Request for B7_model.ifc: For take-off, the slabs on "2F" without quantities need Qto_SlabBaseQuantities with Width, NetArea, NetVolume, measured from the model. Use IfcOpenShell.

First a look at what the model holds.

```python
import ifcopenshell
import ifcopenshell.util.element
import ifcopenshell.util.unit

model = ifcopenshell.open("B7_model.ifc")
print(model.schema)
for unit_type in ("LENGTHUNIT", "AREAUNIT", "VOLUMEUNIT"):
    print(unit_type, ifcopenshell.util.unit.calculate_unit_scale(model, unit_type))
storey = next(s for s in model.by_type("IfcBuildingStorey") if s.Name == "2F")
slabs = [e for e in ifcopenshell.util.element.get_decomposition(storey) if e.is_a("IfcSlab")]
for e in sorted(slabs, key=lambda e: e.id()):
    print(e.id(), e.is_a(), e.Name, list(ifcopenshell.util.element.get_psets(e, qtos_only=True)), sep=" | ")
```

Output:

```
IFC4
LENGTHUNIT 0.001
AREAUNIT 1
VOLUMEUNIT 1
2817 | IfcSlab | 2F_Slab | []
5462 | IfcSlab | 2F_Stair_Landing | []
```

```python
import ifcopenshell
import ifcopenshell.api.pset
import ifcopenshell.geom
import ifcopenshell.util.element
import ifcopenshell.util.shape
import ifcopenshell.util.unit

model = ifcopenshell.open("B7_model.ifc")
unit_scale = ifcopenshell.util.unit.calculate_unit_scale(model)
area_scale = ifcopenshell.util.unit.calculate_unit_scale(model, "AREAUNIT")
volume_scale = ifcopenshell.util.unit.calculate_unit_scale(model, "VOLUMEUNIT")
settings = ifcopenshell.geom.settings()

storey = next(s for s in model.by_type("IfcBuildingStorey") if s.Name == "2F")
slabs = [e for e in ifcopenshell.util.element.get_decomposition(storey) if e.is_a("IfcSlab")]

for e in sorted(slabs, key=lambda e: e.id()):
    if ifcopenshell.util.element.get_psets(e, qtos_only=True, should_inherit=False):
        continue
    # Geometry comes back in metres, in the element's own axes.
    shape = ifcopenshell.geom.create_shape(settings, e)
    values = {
        "Width": ifcopenshell.util.shape.get_z(shape.geometry) / unit_scale,
        "NetArea": ifcopenshell.util.shape.get_footprint_area(shape.geometry) / area_scale,
        "NetVolume": ifcopenshell.util.shape.get_volume(shape.geometry) / volume_scale,
    }
    qto = ifcopenshell.api.pset.add_qto(model, product=e, name="Qto_SlabBaseQuantities")
    ifcopenshell.api.pset.edit_qto(model, qto=qto, properties=values)
    print(e.id(), {k: round(v, 3) for k, v in values.items()})

model.write("B7_model_edited.ifc")
```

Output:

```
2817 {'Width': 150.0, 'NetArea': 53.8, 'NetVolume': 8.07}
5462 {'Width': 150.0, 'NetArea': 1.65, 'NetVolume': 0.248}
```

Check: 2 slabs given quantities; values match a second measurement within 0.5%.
